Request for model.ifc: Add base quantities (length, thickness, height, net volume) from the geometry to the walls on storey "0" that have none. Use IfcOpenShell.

First a look at what the model holds.

```python
import ifcopenshell
import ifcopenshell.util.element
import ifcopenshell.util.unit

model = ifcopenshell.open("model.ifc")
print(model.schema)
for unit_type in ("LENGTHUNIT", "AREAUNIT", "VOLUMEUNIT"):
    print(unit_type, ifcopenshell.util.unit.calculate_unit_scale(model, unit_type))
storey = next(s for s in model.by_type("IfcBuildingStorey") if s.Name == "0")
walls = [e for e in ifcopenshell.util.element.get_decomposition(storey) if e.is_a("IfcWall")]
for e in sorted(walls, key=lambda e: e.id()):
    print(e.id(), e.is_a(), e.Name, list(ifcopenshell.util.element.get_psets(e, qtos_only=True)), sep=" | ")
```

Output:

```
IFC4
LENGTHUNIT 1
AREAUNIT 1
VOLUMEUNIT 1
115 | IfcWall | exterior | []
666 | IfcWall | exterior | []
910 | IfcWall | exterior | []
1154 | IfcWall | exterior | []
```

```python
import ifcopenshell
import ifcopenshell.api.pset
import ifcopenshell.geom
import ifcopenshell.util.element
import ifcopenshell.util.shape
import ifcopenshell.util.unit

model = ifcopenshell.open("model.ifc")
unit_scale = ifcopenshell.util.unit.calculate_unit_scale(model)
volume_scale = ifcopenshell.util.unit.calculate_unit_scale(model, "VOLUMEUNIT")
settings = ifcopenshell.geom.settings()

storey = next(s for s in model.by_type("IfcBuildingStorey") if s.Name == "0")
walls = [e for e in ifcopenshell.util.element.get_decomposition(storey) if e.is_a("IfcWall")]

for e in sorted(walls, key=lambda e: e.id()):
    if ifcopenshell.util.element.get_psets(e, qtos_only=True, should_inherit=False):
        continue
    # Geometry comes back in metres, in the element's own axes.
    shape = ifcopenshell.geom.create_shape(settings, e)
    values = {
        "Length": ifcopenshell.util.shape.get_x(shape.geometry) / unit_scale,
        "Width": ifcopenshell.util.shape.get_y(shape.geometry) / unit_scale,
        "Height": ifcopenshell.util.shape.get_z(shape.geometry) / unit_scale,
        "NetVolume": ifcopenshell.util.shape.get_volume(shape.geometry) / volume_scale,
    }
    qto = ifcopenshell.api.pset.add_qto(model, product=e, name="Qto_WallBaseQuantities")
    ifcopenshell.api.pset.edit_qto(model, qto=qto, properties=values)
    print(e.id(), {k: round(v, 3) for k, v in values.items()})

model.write("model_updated.ifc")
```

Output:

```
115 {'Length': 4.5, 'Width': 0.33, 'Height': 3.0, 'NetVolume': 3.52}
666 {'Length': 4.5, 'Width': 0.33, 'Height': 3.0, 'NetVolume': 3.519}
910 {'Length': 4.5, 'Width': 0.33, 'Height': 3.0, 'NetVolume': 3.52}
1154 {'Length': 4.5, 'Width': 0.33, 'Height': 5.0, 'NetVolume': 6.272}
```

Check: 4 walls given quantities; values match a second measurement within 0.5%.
